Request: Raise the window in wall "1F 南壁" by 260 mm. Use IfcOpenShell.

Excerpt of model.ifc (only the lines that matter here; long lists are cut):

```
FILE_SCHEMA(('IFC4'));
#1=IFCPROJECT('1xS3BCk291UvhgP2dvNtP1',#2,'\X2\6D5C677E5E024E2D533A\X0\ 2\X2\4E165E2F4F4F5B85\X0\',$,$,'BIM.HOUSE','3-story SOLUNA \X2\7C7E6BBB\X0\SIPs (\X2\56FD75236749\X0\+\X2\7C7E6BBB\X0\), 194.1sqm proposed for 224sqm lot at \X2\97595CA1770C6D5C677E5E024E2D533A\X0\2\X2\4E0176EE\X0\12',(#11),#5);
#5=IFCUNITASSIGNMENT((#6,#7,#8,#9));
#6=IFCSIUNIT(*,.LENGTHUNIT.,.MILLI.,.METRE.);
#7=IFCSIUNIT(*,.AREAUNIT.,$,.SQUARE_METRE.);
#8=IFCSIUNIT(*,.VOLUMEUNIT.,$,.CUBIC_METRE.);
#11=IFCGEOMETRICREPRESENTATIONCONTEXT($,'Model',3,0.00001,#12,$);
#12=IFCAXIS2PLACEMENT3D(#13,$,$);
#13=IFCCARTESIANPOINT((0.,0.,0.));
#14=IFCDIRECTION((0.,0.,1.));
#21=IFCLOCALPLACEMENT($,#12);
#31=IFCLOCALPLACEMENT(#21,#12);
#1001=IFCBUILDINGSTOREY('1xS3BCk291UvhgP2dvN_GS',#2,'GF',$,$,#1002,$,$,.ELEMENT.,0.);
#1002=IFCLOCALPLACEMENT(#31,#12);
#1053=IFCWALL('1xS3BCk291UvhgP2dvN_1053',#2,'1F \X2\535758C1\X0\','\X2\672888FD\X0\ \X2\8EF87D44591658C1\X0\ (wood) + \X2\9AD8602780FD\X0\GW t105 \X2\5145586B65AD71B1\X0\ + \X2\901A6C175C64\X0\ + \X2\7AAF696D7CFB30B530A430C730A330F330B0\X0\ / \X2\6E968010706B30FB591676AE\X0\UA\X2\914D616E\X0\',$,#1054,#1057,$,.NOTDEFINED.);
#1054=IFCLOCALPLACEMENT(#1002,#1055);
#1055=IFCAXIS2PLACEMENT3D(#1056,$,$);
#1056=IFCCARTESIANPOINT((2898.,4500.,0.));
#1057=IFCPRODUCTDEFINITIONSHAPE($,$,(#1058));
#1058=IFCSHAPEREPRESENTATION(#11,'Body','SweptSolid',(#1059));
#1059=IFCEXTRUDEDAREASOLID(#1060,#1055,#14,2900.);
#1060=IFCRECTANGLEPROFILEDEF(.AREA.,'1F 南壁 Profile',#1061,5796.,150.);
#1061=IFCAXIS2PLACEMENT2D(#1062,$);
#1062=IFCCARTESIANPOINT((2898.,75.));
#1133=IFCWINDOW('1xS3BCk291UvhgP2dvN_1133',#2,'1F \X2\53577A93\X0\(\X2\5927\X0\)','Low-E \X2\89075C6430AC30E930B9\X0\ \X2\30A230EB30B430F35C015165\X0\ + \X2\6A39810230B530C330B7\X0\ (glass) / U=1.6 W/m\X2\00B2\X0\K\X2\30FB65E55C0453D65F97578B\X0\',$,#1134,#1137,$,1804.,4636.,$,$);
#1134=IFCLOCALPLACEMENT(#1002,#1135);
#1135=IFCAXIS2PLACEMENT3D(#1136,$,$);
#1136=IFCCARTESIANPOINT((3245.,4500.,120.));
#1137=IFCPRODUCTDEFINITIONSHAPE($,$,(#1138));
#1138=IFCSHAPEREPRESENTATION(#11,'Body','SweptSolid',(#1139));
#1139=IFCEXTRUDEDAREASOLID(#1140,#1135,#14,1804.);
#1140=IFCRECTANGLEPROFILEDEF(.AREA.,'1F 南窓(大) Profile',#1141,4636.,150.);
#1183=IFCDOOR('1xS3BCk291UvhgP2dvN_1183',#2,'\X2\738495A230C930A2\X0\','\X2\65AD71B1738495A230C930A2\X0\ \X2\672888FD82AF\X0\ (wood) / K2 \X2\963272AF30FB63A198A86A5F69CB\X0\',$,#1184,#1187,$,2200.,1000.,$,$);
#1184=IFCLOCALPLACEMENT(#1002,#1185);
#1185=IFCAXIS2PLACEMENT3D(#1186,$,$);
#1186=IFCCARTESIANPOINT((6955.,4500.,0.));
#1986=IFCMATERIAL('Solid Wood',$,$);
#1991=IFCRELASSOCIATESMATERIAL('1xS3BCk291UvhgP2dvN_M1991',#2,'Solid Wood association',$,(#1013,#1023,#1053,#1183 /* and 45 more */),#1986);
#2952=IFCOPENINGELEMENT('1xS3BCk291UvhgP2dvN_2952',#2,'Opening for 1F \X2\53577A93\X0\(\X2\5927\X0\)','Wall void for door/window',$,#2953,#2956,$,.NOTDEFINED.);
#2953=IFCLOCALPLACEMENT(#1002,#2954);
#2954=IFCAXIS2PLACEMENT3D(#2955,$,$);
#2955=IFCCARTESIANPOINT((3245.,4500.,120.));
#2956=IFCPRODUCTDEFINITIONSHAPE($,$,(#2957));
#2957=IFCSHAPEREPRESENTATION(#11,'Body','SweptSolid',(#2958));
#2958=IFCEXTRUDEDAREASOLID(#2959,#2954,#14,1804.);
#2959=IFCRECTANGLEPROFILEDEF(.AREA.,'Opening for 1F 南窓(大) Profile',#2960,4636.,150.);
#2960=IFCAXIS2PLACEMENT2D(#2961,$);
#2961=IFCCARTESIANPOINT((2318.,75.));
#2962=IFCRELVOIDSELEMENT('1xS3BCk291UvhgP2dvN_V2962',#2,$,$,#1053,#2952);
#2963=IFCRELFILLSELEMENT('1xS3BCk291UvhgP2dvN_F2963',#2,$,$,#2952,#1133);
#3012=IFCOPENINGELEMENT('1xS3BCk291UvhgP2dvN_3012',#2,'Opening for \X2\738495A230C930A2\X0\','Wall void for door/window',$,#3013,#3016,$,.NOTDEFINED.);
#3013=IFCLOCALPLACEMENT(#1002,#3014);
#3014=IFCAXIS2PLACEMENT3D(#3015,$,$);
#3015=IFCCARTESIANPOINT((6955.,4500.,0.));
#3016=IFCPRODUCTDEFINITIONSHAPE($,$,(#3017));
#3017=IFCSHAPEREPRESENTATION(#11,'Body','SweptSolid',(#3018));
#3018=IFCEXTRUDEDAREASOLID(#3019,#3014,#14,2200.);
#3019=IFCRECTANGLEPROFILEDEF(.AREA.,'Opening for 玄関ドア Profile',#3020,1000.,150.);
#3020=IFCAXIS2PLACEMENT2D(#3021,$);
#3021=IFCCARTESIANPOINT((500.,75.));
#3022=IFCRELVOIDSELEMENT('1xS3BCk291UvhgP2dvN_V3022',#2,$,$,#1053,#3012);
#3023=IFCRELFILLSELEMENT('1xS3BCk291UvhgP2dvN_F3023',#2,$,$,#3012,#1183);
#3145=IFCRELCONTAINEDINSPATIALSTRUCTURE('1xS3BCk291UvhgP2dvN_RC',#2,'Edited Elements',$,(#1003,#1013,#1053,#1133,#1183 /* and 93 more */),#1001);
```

```python
import numpy as np
import ifcopenshell
import ifcopenshell.api.geometry
import ifcopenshell.util.placement
import ifcopenshell.util.unit

model = ifcopenshell.open("model.ifc")
unit_scale = ifcopenshell.util.unit.calculate_unit_scale(model)

window = model.by_guid("1xS3BCk291UvhgP2dvN_1133")
opening = window.FillsVoids[0].RelatingOpeningElement
dz = 0.26 / unit_scale

shift = np.array([0.0, 0.0, dz])
# The window is not placed relative to its opening, so move both.
for product in (opening, window):
    matrix = ifcopenshell.util.placement.get_local_placement(product.ObjectPlacement)
    matrix[:3, 3] += shift
    ifcopenshell.api.geometry.edit_object_placement(model, product=product, matrix=matrix, is_si=False)

print(f"moved by {dz * unit_scale:+.3f} m")

model.write("model_v2.ifc")
```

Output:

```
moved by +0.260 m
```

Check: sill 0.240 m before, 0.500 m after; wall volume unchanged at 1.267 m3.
